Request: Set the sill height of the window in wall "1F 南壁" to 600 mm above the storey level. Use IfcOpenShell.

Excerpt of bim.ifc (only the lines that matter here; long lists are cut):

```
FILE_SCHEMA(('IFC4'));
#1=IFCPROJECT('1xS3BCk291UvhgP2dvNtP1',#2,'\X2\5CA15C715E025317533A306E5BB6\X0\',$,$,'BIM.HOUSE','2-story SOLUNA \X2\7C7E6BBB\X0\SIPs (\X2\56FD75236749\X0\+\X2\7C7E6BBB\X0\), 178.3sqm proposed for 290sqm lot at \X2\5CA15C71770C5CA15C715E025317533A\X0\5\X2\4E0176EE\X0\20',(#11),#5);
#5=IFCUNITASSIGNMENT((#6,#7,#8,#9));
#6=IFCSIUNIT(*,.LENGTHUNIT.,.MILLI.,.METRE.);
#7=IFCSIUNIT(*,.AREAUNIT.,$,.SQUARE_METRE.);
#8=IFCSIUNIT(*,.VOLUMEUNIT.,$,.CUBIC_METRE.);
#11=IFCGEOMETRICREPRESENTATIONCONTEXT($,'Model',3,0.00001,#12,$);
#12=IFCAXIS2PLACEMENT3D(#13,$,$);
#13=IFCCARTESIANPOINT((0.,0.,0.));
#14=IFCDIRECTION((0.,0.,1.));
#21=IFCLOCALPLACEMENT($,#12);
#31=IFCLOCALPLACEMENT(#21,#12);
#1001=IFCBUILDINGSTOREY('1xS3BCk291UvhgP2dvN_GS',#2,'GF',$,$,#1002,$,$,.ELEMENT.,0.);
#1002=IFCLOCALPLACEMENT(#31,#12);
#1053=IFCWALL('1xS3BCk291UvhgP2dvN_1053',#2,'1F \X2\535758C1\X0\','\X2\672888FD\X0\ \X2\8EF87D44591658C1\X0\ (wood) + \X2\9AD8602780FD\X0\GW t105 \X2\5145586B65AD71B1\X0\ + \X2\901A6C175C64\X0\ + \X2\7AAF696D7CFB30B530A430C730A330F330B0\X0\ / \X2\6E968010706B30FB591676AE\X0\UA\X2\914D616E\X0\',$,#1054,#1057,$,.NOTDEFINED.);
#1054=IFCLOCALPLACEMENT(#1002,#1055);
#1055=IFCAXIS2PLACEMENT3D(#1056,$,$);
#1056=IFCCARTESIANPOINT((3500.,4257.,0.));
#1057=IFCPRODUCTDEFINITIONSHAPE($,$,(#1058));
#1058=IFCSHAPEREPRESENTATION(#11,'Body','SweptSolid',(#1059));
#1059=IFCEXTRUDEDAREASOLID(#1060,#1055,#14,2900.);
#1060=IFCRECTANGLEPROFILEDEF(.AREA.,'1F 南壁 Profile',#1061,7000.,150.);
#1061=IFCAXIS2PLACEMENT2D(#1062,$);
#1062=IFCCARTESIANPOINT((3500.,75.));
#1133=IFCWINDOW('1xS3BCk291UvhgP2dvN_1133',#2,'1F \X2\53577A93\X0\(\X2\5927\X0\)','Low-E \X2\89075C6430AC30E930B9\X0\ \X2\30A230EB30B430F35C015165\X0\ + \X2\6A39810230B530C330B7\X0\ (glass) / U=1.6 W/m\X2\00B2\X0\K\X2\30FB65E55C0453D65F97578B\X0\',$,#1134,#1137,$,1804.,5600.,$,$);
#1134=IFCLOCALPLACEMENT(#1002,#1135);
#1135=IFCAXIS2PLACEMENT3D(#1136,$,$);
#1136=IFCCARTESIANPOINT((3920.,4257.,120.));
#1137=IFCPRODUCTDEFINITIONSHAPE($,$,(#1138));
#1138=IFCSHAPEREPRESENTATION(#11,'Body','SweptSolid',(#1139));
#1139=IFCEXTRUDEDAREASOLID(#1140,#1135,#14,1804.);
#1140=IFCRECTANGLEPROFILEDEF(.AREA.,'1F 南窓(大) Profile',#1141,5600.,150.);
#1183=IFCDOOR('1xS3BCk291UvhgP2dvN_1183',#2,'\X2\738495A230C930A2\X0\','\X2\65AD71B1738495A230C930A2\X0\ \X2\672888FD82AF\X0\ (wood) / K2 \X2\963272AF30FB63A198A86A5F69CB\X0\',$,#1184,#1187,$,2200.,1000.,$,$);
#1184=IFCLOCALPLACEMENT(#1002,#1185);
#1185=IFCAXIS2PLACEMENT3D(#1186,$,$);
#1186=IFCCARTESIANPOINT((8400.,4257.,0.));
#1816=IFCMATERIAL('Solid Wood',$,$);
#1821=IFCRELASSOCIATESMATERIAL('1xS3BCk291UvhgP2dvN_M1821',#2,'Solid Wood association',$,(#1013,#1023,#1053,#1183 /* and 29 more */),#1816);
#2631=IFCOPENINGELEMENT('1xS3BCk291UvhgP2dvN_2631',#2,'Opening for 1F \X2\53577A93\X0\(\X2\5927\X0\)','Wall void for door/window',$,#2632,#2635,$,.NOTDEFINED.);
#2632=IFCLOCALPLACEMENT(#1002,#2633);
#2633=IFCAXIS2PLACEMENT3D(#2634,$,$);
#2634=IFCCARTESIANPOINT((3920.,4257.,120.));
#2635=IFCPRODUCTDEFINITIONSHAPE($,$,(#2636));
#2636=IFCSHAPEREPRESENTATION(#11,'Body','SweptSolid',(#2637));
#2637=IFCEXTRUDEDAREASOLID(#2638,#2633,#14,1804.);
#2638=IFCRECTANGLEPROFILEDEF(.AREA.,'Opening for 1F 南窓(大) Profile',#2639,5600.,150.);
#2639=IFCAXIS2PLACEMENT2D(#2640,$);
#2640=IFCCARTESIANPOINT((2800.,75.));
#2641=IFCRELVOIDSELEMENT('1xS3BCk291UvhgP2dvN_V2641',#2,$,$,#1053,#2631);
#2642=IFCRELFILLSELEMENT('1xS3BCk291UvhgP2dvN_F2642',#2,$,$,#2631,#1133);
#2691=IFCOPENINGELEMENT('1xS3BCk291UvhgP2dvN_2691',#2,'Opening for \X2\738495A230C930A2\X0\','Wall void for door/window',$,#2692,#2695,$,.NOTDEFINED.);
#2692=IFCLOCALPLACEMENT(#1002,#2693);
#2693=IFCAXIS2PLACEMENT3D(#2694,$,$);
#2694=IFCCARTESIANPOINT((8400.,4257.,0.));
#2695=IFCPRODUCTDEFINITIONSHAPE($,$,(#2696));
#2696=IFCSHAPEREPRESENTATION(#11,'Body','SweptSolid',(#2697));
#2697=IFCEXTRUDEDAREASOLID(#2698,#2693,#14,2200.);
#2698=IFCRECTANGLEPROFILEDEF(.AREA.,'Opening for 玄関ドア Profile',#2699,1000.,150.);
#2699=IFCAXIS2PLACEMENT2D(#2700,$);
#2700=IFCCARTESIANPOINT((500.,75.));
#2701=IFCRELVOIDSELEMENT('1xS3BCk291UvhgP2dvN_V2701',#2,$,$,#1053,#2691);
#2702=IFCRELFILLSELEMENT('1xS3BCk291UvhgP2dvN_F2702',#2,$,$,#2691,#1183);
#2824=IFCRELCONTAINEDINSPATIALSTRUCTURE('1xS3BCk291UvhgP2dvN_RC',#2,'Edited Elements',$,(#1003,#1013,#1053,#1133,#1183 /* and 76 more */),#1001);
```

```python
import numpy as np
import ifcopenshell
import ifcopenshell.api.geometry
import ifcopenshell.geom
import ifcopenshell.util.element
import ifcopenshell.util.placement
import ifcopenshell.util.shape
import ifcopenshell.util.unit

model = ifcopenshell.open("bim.ifc")
unit_scale = ifcopenshell.util.unit.calculate_unit_scale(model)

window = model.by_guid("1xS3BCk291UvhgP2dvN_1133")
opening = window.FillsVoids[0].RelatingOpeningElement
storey = ifcopenshell.util.element.get_container(window, ifc_class="IfcBuildingStorey")
level = ifcopenshell.util.placement.get_local_placement(storey.ObjectPlacement)[2, 3]

# The opening's origin need not be at the sill, so measure its lowest point.
shape = ifcopenshell.geom.create_shape(ifcopenshell.geom.settings(), opening)
bottom = ifcopenshell.util.shape.get_shape_bottom_elevation(shape, shape.geometry) / unit_scale
dz = level + 0.6 / unit_scale - bottom

shift = np.array([0.0, 0.0, dz])
# The window is not placed relative to its opening, so move both.
for product in (opening, window):
    matrix = ifcopenshell.util.placement.get_local_placement(product.ObjectPlacement)
    matrix[:3, 3] += shift
    ifcopenshell.api.geometry.edit_object_placement(model, product=product, matrix=matrix, is_si=False)

print(f"moved by {dz * unit_scale:+.3f} m")

model.write("bim_rev.ifc")
```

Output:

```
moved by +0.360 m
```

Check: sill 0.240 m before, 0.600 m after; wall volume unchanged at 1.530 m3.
